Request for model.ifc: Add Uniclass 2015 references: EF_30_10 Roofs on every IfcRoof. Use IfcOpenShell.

First a look at what the model holds.

```python
import ifcopenshell

model = ifcopenshell.open("model.ifc")
print(model.schema)
print("classifications:", [c.Name for c in model.by_type("IfcClassification")])
for ifc_class in ("IfcDoor", "IfcRoof", "IfcStair", "IfcWall", "IfcWindow"):
    print(ifc_class, len(model.by_type(ifc_class)))
```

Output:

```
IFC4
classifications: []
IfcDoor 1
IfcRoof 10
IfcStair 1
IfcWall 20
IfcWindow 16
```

```python
import ifcopenshell
import ifcopenshell.api.classification

model = ifcopenshell.open("model.ifc")

system = ifcopenshell.api.classification.add_classification(model, classification="Uniclass 2015")

codes = {
    "IfcRoof": ("EF_30_10", "Roofs"),
}
for ifc_class, (code, name) in codes.items():
    products = model.by_type(ifc_class)
    ifcopenshell.api.classification.add_reference(
        model, products=products, classification=system, identification=code, name=name
    )
    print(code, len(products))

model.write("model_edited.ifc")
```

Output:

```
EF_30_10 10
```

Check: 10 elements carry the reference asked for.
